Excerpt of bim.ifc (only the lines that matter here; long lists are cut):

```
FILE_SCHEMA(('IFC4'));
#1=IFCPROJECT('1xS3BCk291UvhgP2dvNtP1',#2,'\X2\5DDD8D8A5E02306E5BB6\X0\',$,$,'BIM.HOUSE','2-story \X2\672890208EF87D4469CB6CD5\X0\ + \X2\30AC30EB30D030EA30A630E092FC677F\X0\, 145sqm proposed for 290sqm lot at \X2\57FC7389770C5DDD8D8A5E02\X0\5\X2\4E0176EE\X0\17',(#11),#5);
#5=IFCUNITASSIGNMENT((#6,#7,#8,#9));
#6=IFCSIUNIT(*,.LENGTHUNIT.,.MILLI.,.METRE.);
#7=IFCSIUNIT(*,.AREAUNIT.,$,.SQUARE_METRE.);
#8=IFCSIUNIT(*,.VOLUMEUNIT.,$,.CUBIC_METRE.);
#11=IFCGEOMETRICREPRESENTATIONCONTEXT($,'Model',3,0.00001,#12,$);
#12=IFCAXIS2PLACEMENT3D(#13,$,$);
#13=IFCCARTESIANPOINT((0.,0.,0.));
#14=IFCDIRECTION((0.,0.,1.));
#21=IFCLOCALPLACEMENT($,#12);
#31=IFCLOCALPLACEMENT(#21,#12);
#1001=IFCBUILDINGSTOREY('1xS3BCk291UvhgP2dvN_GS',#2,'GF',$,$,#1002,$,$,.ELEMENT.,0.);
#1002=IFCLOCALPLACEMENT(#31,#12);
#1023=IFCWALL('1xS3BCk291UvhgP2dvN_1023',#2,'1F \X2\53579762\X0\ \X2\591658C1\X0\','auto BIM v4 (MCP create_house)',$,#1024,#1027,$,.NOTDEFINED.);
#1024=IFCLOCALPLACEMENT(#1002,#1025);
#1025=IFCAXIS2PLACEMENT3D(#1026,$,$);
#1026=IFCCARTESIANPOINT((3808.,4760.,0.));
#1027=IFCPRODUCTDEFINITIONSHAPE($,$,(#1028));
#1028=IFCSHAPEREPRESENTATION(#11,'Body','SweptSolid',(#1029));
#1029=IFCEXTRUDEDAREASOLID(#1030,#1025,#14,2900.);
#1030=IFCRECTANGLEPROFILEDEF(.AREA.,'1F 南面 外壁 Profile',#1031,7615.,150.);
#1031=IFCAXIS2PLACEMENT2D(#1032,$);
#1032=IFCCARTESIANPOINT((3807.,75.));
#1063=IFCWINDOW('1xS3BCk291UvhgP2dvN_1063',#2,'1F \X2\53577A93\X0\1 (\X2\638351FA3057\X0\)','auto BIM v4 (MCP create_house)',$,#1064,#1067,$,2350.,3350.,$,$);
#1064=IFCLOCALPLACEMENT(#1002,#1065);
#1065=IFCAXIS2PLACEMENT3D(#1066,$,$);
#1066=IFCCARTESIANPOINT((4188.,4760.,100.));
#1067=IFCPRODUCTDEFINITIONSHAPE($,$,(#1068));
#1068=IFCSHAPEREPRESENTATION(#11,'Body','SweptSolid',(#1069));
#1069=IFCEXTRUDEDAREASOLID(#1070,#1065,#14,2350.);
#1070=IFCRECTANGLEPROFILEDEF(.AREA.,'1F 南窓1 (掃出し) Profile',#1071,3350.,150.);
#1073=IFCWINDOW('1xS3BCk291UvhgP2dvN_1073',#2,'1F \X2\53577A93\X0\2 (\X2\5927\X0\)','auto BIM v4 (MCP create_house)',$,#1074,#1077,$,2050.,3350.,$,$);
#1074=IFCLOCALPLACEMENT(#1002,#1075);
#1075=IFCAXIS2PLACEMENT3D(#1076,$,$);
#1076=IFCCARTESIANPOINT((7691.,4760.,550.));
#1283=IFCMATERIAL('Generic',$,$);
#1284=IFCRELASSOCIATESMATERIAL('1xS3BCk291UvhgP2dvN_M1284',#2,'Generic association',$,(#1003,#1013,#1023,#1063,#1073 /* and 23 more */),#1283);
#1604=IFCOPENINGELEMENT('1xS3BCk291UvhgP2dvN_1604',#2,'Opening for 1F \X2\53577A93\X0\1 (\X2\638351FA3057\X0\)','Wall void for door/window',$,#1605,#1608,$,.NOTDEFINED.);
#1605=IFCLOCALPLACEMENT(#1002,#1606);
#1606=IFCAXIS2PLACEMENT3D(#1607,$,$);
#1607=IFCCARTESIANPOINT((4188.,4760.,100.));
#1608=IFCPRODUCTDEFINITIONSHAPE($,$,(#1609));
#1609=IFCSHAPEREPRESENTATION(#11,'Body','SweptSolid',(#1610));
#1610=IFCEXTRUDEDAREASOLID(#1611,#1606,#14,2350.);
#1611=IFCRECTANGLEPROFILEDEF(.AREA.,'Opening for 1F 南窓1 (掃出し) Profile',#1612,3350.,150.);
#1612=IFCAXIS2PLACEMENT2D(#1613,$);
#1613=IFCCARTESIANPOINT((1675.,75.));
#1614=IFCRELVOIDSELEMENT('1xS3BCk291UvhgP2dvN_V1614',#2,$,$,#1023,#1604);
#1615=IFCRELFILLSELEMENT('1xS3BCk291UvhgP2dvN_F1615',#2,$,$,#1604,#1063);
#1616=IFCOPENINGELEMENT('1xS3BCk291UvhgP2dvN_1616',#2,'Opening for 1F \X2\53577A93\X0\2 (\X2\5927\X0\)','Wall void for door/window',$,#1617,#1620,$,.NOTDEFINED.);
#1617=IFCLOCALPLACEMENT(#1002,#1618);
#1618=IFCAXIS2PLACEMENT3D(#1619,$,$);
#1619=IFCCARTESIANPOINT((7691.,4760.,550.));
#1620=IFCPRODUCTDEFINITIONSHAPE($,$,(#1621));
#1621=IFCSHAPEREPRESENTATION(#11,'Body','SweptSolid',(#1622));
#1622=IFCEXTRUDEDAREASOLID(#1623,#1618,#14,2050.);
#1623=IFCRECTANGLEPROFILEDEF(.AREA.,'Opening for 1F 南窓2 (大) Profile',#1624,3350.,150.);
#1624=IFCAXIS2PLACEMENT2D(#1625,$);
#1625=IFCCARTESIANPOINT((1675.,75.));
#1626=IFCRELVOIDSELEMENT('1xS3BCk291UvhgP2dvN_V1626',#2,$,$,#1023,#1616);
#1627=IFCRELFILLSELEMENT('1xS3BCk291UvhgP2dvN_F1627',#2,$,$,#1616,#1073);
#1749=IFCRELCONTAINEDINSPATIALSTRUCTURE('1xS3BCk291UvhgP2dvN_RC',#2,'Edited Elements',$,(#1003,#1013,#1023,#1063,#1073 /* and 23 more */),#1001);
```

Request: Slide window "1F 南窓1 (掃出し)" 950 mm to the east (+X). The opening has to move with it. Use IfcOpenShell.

```python
import ifcopenshell
import ifcopenshell.api.geometry
import ifcopenshell.util.placement

model = ifcopenshell.open("bim.ifc")

window = model.by_guid("1xS3BCk291UvhgP2dvN_1063")
opening = window.FillsVoids[0].RelatingOpeningElement
wall = opening.VoidsElements[0].RelatingBuildingElement

wall_matrix = ifcopenshell.util.placement.get_local_placement(wall.ObjectPlacement)
shift = wall_matrix[:3, 0] * 950.0
before = ifcopenshell.util.placement.get_local_placement(window.ObjectPlacement)[:3, 3].copy()

# The window is not placed relative to its opening, so move both.
for product in (opening, window):
    matrix = ifcopenshell.util.placement.get_local_placement(product.ObjectPlacement)
    matrix[:3, 3] += shift
    ifcopenshell.api.geometry.edit_object_placement(model, product=product, matrix=matrix, is_si=False)

after = ifcopenshell.util.placement.get_local_placement(window.ObjectPlacement)[:3, 3]
print("window moved by", (after - before).round(3) + 0.0)

model.write("bim_updated.ifc")
```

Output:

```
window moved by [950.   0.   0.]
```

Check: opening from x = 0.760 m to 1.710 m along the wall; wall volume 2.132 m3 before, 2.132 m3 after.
